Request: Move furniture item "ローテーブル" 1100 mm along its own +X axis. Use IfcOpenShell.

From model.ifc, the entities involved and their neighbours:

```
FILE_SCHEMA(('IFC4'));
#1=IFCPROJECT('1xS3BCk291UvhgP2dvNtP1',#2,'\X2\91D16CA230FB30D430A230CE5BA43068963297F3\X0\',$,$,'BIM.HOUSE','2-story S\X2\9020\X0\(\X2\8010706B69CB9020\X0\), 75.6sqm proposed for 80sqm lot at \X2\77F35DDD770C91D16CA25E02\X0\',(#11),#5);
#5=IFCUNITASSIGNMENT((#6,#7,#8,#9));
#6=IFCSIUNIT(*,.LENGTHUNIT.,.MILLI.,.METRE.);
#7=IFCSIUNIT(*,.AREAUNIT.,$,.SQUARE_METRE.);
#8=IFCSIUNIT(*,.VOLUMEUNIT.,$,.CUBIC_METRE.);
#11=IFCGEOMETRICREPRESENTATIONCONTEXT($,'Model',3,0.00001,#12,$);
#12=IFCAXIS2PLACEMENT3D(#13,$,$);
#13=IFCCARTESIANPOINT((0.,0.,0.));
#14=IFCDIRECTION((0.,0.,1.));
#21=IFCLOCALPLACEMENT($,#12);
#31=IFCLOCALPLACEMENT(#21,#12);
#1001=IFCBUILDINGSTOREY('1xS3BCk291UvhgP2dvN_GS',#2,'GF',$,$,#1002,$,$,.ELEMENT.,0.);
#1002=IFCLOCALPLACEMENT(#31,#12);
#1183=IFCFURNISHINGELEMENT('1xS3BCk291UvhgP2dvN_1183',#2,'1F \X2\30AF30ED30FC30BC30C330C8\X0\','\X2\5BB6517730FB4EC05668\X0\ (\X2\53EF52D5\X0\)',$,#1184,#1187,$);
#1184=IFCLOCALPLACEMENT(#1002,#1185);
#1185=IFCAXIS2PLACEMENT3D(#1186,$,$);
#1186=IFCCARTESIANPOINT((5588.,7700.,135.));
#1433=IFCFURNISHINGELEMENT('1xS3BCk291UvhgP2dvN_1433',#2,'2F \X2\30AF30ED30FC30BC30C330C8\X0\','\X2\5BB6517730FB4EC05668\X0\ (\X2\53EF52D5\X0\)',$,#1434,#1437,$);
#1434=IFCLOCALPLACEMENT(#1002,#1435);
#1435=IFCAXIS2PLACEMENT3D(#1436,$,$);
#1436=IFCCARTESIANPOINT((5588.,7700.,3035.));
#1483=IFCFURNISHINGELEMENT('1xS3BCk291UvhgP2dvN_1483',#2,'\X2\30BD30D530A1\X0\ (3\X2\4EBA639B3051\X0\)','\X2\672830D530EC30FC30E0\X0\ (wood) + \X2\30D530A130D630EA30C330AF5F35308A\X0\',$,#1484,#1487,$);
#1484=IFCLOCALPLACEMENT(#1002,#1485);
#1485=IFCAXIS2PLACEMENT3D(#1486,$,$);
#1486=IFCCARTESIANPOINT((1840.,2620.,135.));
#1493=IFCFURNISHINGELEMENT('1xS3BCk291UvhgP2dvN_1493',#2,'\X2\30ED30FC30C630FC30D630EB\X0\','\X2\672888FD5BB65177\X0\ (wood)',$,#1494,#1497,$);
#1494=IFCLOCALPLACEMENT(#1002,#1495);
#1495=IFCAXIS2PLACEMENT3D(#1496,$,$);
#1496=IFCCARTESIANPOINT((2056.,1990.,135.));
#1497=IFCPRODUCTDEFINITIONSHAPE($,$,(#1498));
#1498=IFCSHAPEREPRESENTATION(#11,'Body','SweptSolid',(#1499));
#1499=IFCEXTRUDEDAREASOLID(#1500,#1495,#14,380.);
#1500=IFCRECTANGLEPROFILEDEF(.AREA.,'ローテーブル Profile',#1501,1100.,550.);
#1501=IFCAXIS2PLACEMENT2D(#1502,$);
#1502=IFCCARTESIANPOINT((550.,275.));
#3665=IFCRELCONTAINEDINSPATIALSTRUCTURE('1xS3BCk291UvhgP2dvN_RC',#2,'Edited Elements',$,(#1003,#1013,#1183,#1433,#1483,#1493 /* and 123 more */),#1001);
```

```python
import ifcopenshell
import ifcopenshell.api.geometry
import ifcopenshell.util.placement

model = ifcopenshell.open("model.ifc")

item = model.by_guid("1xS3BCk291UvhgP2dvN_1493")
matrix = ifcopenshell.util.placement.get_local_placement(item.ObjectPlacement)
matrix[:3, 3] += matrix[:3, 0] * 1100.0
ifcopenshell.api.geometry.edit_object_placement(model, product=item, matrix=matrix, is_si=False)

print(ifcopenshell.util.placement.get_local_placement(item.ObjectPlacement).round(3) + 0.0)

model.write("model_updated.ifc")
```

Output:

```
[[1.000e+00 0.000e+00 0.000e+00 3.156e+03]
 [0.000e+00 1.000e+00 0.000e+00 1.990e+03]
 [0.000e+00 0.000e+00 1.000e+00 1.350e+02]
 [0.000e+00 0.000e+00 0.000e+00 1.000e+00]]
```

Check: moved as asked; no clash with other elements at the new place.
